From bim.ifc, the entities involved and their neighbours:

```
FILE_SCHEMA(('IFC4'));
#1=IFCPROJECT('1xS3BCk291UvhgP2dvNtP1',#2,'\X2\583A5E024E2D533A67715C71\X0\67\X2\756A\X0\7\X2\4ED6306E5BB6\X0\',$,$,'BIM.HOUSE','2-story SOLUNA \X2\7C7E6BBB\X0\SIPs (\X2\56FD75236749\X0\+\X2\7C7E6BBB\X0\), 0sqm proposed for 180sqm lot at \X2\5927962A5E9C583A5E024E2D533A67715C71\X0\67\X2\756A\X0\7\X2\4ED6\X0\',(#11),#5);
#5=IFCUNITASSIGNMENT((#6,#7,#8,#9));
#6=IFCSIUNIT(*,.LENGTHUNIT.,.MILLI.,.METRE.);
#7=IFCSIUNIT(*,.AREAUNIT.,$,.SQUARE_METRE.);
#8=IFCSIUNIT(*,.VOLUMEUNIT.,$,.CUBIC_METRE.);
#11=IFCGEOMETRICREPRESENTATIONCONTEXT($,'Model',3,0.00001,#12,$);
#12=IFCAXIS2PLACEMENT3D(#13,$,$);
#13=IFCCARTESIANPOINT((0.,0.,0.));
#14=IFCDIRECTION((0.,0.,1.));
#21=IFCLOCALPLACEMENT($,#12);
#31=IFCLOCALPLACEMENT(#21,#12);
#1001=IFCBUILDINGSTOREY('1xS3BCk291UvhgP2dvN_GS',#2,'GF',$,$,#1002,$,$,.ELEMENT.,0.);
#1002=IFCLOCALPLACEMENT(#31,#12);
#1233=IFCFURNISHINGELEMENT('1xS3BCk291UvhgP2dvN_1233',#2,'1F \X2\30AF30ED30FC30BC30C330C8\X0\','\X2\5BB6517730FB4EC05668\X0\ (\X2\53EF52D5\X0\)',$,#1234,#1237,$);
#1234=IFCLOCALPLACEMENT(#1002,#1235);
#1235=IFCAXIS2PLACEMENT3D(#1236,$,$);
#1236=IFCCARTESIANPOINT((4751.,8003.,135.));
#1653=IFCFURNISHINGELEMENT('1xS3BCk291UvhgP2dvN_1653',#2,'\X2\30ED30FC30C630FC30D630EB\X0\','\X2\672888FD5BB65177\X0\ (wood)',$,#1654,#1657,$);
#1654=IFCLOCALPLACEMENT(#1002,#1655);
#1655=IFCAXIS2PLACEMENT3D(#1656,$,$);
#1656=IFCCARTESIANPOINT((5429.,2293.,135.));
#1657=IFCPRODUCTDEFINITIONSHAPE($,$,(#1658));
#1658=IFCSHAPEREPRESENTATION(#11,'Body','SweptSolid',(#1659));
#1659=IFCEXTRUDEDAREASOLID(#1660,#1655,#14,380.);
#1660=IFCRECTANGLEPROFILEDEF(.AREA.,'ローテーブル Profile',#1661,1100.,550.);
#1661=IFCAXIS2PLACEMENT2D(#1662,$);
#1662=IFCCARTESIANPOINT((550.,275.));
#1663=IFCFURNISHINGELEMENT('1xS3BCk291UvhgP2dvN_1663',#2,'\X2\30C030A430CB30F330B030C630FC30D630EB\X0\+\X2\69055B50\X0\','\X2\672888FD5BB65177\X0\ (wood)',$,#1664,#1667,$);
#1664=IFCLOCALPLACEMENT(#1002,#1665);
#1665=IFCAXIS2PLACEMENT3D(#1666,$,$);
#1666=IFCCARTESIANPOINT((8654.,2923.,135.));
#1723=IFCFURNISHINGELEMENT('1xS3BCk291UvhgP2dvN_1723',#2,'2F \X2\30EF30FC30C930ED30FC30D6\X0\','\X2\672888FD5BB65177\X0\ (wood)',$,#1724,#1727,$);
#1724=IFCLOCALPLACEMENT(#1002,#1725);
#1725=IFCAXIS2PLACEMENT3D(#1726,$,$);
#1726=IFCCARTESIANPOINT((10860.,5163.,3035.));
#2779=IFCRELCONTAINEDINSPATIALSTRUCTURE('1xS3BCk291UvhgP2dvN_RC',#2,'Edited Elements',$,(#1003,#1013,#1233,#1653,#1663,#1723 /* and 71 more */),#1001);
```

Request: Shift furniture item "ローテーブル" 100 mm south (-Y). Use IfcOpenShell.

```python
import ifcopenshell
import ifcopenshell.api.geometry
import ifcopenshell.util.placement
import ifcopenshell.util.unit

model = ifcopenshell.open("bim.ifc")
unit_scale = ifcopenshell.util.unit.calculate_unit_scale(model)

item = model.by_guid("1xS3BCk291UvhgP2dvN_1653")
matrix = ifcopenshell.util.placement.get_local_placement(item.ObjectPlacement)
matrix[1, 3] -= 0.1 / unit_scale
ifcopenshell.api.geometry.edit_object_placement(model, product=item, matrix=matrix, is_si=False)

print(ifcopenshell.util.placement.get_local_placement(item.ObjectPlacement).round(3) + 0.0)

model.write("bim_v2.ifc")
```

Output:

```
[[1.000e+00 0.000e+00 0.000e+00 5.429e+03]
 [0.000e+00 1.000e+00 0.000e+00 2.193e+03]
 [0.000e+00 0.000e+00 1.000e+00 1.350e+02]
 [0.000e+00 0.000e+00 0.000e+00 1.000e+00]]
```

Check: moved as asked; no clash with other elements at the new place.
